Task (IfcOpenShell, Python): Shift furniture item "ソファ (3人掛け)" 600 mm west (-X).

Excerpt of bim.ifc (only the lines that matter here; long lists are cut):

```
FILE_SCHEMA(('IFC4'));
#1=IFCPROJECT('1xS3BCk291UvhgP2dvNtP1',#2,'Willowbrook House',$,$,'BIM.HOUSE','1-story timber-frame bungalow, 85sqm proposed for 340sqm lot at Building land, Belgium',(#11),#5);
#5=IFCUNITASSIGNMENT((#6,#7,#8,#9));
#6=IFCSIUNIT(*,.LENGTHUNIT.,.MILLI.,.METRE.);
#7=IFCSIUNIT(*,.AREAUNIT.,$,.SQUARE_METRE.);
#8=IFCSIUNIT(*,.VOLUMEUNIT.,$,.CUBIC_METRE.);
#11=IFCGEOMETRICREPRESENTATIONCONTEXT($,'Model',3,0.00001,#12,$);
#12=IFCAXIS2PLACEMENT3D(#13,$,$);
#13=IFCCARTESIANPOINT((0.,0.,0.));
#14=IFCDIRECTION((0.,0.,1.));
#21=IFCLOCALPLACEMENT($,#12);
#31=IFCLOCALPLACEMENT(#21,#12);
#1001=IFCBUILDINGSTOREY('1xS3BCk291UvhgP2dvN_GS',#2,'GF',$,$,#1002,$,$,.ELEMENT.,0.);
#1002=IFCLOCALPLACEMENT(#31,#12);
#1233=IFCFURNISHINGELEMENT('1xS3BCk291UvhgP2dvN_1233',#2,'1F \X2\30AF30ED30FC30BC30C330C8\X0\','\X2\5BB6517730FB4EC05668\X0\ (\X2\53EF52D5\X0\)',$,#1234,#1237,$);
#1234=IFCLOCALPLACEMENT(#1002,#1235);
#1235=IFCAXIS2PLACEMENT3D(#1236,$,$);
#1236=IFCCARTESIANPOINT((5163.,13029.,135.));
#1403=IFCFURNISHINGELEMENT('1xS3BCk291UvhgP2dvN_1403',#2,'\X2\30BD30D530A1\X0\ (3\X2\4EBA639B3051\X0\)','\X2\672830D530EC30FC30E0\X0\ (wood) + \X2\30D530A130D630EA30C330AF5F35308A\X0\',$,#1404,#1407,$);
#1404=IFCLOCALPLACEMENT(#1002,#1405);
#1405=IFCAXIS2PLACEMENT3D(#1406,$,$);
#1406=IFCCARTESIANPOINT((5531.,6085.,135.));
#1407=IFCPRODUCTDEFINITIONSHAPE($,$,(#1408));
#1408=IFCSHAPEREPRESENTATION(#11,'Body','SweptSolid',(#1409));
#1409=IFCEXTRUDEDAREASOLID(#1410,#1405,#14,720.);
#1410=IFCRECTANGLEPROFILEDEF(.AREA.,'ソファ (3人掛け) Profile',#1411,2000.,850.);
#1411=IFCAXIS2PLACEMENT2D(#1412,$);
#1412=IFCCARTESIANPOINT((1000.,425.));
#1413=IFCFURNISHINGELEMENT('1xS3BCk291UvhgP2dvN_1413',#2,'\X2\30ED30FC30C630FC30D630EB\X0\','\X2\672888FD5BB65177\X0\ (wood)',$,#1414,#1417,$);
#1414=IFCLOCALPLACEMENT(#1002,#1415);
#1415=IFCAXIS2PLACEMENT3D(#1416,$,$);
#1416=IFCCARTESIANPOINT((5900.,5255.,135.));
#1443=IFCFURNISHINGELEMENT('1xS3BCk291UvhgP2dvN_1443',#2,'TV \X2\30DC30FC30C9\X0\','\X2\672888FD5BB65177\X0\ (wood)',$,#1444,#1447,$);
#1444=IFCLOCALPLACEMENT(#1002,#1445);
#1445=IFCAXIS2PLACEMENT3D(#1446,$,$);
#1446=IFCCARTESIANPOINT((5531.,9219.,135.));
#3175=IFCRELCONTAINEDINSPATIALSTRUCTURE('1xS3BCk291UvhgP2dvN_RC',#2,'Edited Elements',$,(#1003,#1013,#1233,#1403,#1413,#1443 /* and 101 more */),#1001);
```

```python
import ifcopenshell
import ifcopenshell.api.geometry
import ifcopenshell.util.placement

model = ifcopenshell.open("bim.ifc")

item = model.by_guid("1xS3BCk291UvhgP2dvN_1403")
matrix = ifcopenshell.util.placement.get_local_placement(item.ObjectPlacement)
matrix[0, 3] -= 600.0
ifcopenshell.api.geometry.edit_object_placement(model, product=item, matrix=matrix, is_si=False)

print(ifcopenshell.util.placement.get_local_placement(item.ObjectPlacement).round(3) + 0.0)

model.write("bim_rev.ifc")
```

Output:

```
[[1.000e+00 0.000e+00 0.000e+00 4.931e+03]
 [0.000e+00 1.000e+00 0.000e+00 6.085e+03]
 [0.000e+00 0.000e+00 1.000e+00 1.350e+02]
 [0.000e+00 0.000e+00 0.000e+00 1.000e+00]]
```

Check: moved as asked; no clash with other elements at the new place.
